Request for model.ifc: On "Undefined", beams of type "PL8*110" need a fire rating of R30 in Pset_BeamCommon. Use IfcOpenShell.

First a look at what the model holds.

```python
import ifcopenshell
import ifcopenshell.util.element

model = ifcopenshell.open("model.ifc")
print(model.schema)
storey = next(s for s in model.by_type("IfcBuildingStorey") if s.Name == "Undefined")
beams = [e for e in ifcopenshell.util.element.get_decomposition(storey) if e.is_a("IfcBeam")]
seen = {}
for e in beams:
    element_type = ifcopenshell.util.element.get_type(e)
    key = (element_type.Name if element_type != e and element_type else None, ifcopenshell.util.element.get_pset(e, "Pset_BeamCommon", "FireRating"))
    seen[key] = seen.get(key, 0) + 1
for (name, value), count in sorted(seen.items(), key=str):
    print(count, "x", name, "|", value)
```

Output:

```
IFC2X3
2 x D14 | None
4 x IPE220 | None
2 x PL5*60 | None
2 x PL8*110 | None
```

```python
import ifcopenshell
import ifcopenshell.api.pset
import ifcopenshell.util.element

model = ifcopenshell.open("model.ifc")

storey = next(s for s in model.by_type("IfcBuildingStorey") if s.Name == "Undefined")
beams = [e for e in ifcopenshell.util.element.get_decomposition(storey) if e.is_a("IfcBeam")]

count = 0
for e in beams:
    element_type = ifcopenshell.util.element.get_type(e)
    if element_type in (None, e) or element_type.Name != "PL8*110":
        continue
    found = ifcopenshell.util.element.get_pset(e, "Pset_BeamCommon", should_inherit=False)
    if found:
        pset = model.by_id(found["id"])
        if len(ifcopenshell.util.element.get_elements_by_pset(pset)) > 1:
            pset = ifcopenshell.api.pset.unshare_pset(model, products=[e], pset=pset)[0]
    else:
        pset = ifcopenshell.api.pset.add_pset(model, product=e, name="Pset_BeamCommon")
    ifcopenshell.api.pset.edit_pset(model, pset=pset, properties={"FireRating": "R30"})
    count += 1

print(count, "beams updated")

model.write("model_updated.ifc")
```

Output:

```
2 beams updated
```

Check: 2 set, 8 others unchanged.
